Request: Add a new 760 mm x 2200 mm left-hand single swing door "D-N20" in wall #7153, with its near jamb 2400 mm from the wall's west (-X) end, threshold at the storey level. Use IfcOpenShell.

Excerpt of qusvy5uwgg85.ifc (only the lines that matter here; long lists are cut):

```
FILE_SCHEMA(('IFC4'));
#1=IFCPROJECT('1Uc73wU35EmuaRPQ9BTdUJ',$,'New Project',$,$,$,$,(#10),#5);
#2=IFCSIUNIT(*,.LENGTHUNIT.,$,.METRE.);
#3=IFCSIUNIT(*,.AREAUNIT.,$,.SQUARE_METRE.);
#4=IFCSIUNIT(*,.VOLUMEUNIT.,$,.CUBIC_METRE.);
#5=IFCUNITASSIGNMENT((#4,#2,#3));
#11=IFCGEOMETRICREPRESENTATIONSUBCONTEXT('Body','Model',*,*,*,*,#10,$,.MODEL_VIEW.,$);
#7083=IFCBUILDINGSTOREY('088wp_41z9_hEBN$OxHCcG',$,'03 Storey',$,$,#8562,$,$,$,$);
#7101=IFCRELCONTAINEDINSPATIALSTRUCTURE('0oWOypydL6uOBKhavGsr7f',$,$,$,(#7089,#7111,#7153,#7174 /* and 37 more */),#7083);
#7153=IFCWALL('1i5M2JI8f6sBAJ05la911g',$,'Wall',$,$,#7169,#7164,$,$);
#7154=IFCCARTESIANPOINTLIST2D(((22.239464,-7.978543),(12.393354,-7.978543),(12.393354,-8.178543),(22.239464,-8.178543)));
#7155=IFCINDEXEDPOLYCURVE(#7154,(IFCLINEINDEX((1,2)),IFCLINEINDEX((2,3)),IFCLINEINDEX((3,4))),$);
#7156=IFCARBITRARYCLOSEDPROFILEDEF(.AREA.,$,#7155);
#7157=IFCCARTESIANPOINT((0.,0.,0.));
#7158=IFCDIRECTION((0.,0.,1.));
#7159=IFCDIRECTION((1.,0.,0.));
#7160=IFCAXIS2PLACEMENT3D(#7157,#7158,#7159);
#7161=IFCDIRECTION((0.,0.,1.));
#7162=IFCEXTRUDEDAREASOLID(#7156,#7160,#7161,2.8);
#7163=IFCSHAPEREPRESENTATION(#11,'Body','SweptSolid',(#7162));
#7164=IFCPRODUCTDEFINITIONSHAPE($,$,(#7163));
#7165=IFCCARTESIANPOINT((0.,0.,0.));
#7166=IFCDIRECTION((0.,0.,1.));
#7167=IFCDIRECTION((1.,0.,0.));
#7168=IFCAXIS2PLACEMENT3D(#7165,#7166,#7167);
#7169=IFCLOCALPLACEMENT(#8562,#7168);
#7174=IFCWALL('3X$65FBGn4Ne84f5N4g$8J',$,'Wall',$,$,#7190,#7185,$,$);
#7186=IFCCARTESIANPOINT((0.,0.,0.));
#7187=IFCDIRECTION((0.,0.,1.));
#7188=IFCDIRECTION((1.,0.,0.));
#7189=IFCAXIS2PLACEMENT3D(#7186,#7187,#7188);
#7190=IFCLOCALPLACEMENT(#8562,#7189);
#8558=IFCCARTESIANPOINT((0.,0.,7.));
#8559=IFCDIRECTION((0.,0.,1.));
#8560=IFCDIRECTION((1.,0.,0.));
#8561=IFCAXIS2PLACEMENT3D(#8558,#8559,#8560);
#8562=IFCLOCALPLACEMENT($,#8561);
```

```python
import numpy as np
import ifcopenshell
import ifcopenshell.api.feature
import ifcopenshell.api.geometry
import ifcopenshell.api.root
import ifcopenshell.api.spatial
import ifcopenshell.geom
import ifcopenshell.util.element
import ifcopenshell.util.placement
import ifcopenshell.util.representation
import ifcopenshell.util.shape
import ifcopenshell.util.unit

model = ifcopenshell.open("qusvy5uwgg85.ifc")
unit_scale = ifcopenshell.util.unit.calculate_unit_scale(model)
settings = ifcopenshell.geom.settings()


def volume(element):
    """Net volume in cubic metres, openings subtracted."""
    shape = ifcopenshell.geom.create_shape(settings, element)
    return ifcopenshell.util.shape.get_volume(shape.geometry)


wall = model.by_guid("1i5M2JI8f6sBAJ05la911g")
storey = ifcopenshell.util.element.get_container(wall, ifc_class="IfcBuildingStorey")
context = ifcopenshell.util.representation.get_context(model, "Model", "Body", "MODEL_VIEW")
before = volume(wall)

width, height, from_end, sill = 0.76, 2.2, 2.4, 0.0  # metres

# The wall runs along its own X axis, and the end named is its -X end.
wall_shape = ifcopenshell.geom.create_shape(settings, wall)
x, y, z = ifcopenshell.util.shape.get_vertices(wall_shape.geometry).T
start = x.min() + from_end
face, thickness = float(y.min()), float(y.max() - y.min())
wall_matrix = ifcopenshell.util.placement.get_local_placement(wall.ObjectPlacement)
level = ifcopenshell.util.placement.get_local_placement(storey.ObjectPlacement)[2, 3]


def in_wall(x, y):
    """Placement at x, y metres in the wall's axes, at sill height."""
    matrix = wall_matrix.copy()
    matrix[:, 3] = wall_matrix @ np.array([x / unit_scale, y / unit_scale, 0.0, 1.0])
    matrix[2, 3] = level + sill / unit_scale
    return matrix


# Opening: a box that overshoots both wall faces by 50 mm.
opening = ifcopenshell.api.root.create_entity(model, ifc_class="IfcOpeningElement", predefined_type="OPENING")
box = ifcopenshell.api.geometry.add_wall_representation(
    model, context=context, length=width, height=height, thickness=thickness + 0.1
)
ifcopenshell.api.geometry.assign_representation(model, product=opening, representation=box)
ifcopenshell.api.geometry.edit_object_placement(model, product=opening, matrix=in_wall(start, face - 0.05), is_si=False)
ifcopenshell.api.feature.add_feature(model, feature=opening, element=wall)

door = ifcopenshell.api.root.create_entity(model, ifc_class="IfcDoor", name="D-N20", predefined_type="DOOR")
door.OverallWidth, door.OverallHeight = width / unit_scale, height / unit_scale
door.OperationType = "SINGLE_SWING_LEFT"
body = ifcopenshell.api.geometry.add_door_representation(
    model,
    context=context,
    overall_width=door.OverallWidth,
    overall_height=door.OverallHeight,
    operation_type="SINGLE_SWING_LEFT",
    lining_properties={"LiningDepth": thickness / unit_scale, "ThresholdDepth": thickness / unit_scale},
)
ifcopenshell.api.geometry.assign_representation(model, product=door, representation=body)
ifcopenshell.api.spatial.assign_container(model, products=[door], relating_structure=storey)
ifcopenshell.api.feature.add_filling(model, opening=opening, element=door)

# The lining spans the wall, so the door starts at the wall face.
ifcopenshell.api.geometry.edit_object_placement(model, product=door, matrix=in_wall(start, face), is_si=False)

after = volume(wall)

print(f"wall volume {before:.3f} -> {after:.3f} m3")

model.write("qusvy5uwgg85_rev.ifc")
```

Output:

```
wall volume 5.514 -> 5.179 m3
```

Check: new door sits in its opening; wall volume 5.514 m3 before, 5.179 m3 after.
